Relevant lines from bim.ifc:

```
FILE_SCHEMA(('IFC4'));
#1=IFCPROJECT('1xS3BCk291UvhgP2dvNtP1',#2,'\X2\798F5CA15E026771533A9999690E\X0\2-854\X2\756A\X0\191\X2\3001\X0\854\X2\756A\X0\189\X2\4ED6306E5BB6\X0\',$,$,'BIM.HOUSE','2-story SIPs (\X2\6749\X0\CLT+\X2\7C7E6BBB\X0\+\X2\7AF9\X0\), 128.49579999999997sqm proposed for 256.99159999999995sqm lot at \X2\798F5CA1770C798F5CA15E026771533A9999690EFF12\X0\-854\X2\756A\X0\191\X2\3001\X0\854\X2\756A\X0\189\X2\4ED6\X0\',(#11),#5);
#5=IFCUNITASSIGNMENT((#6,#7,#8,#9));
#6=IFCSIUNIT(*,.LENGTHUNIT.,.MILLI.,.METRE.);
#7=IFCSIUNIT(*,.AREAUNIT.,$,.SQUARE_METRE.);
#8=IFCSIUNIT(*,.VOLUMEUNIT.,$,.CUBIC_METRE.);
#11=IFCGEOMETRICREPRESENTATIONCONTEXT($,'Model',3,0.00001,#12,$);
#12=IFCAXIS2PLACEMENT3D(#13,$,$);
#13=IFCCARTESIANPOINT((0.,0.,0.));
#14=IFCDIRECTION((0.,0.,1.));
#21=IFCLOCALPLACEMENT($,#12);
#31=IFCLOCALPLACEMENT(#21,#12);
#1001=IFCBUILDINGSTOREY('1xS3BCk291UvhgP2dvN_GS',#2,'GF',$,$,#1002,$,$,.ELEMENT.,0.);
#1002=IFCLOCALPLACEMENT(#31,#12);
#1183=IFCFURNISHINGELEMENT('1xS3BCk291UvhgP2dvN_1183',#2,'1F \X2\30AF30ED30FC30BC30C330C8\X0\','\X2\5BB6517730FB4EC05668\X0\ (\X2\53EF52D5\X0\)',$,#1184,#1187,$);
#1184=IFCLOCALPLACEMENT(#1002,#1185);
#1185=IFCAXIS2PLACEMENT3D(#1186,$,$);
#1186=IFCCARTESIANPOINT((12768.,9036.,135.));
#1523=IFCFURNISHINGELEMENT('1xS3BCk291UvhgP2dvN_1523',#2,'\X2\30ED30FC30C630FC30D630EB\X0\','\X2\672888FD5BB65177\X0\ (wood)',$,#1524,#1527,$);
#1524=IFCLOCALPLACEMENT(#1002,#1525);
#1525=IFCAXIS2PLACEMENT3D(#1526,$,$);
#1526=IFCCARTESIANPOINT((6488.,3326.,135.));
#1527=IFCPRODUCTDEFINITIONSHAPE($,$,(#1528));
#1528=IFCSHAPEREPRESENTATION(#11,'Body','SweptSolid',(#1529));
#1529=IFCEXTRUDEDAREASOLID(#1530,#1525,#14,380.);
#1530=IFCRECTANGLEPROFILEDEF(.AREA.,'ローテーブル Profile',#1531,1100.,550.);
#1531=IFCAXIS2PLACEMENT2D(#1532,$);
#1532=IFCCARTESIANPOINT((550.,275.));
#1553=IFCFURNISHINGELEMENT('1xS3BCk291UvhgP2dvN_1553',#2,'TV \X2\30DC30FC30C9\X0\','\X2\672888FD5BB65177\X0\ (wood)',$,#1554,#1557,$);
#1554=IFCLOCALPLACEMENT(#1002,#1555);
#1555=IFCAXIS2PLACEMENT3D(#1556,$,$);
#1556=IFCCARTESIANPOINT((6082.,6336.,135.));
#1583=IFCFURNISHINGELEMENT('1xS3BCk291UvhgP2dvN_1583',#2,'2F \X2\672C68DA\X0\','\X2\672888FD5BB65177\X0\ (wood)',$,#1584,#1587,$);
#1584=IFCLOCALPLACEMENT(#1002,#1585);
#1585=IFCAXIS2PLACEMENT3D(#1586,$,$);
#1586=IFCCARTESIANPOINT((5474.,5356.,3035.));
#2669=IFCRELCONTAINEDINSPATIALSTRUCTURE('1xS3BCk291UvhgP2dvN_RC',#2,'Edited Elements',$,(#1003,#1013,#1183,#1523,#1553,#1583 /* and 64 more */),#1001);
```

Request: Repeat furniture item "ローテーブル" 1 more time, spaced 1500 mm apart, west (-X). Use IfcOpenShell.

```python
import numpy as np
import ifcopenshell
import ifcopenshell.api.geometry
import ifcopenshell.api.root
import ifcopenshell.util.element
import ifcopenshell.util.placement

model = ifcopenshell.open("bim.ifc")


def reuse_history(source, copy):
    """copy_class also copies each property set's owner history, people and application; keep the originals."""
    for rel in copy.IsDefinedBy:
        if rel.is_a("IfcRelDefinesByProperties") and (history := rel.RelatingPropertyDefinition.OwnerHistory):
            rel.RelatingPropertyDefinition.OwnerHistory = source.OwnerHistory
            ifcopenshell.util.element.remove_deep2(model, history)


source = model.by_guid("1xS3BCk291UvhgP2dvN_1523")
base = ifcopenshell.util.placement.get_local_placement(source.ObjectPlacement)
step = np.array([-1.0, 0.0, 0.0]) * 1500.0

for i in range(1, 2):
    copy = ifcopenshell.api.root.copy_class(model, product=source)
    copy.Representation = ifcopenshell.util.element.copy_deep(
        model, source.Representation, exclude=["IfcGeometricRepresentationContext", "IfcRepresentationMap"]
    )
    reuse_history(source, copy)
    matrix = base.copy()
    matrix[:3, 3] += i * step
    print("added at", matrix[:3, 3].round(3) + 0.0)
    ifcopenshell.api.geometry.edit_object_placement(model, product=copy, matrix=matrix, is_si=False)

model.write("bim-out.ifc")
```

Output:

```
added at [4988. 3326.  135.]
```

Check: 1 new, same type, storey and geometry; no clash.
